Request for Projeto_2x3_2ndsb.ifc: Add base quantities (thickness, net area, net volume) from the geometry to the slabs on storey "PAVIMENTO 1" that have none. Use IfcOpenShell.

First a look at what the model holds.

```python
import ifcopenshell
import ifcopenshell.util.element
import ifcopenshell.util.unit

model = ifcopenshell.open("Projeto_2x3_2ndsb.ifc")
print(model.schema)
for unit_type in ("LENGTHUNIT", "AREAUNIT", "VOLUMEUNIT"):
    print(unit_type, ifcopenshell.util.unit.calculate_unit_scale(model, unit_type))
storey = next(s for s in model.by_type("IfcBuildingStorey") if s.Name == "PAVIMENTO 1")
slabs = [e for e in ifcopenshell.util.element.get_decomposition(storey) if e.is_a("IfcSlab")]
for e in sorted(slabs, key=lambda e: e.id()):
    print(e.id(), e.is_a(), e.Name, list(ifcopenshell.util.element.get_psets(e, qtos_only=True)), sep=" | ")
```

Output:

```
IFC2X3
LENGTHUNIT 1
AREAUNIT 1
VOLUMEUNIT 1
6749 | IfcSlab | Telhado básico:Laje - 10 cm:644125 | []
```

```python
import ifcopenshell
import ifcopenshell.api.pset
import ifcopenshell.geom
import ifcopenshell.util.element
import ifcopenshell.util.shape
import ifcopenshell.util.unit

model = ifcopenshell.open("Projeto_2x3_2ndsb.ifc")
unit_scale = ifcopenshell.util.unit.calculate_unit_scale(model)
area_scale = ifcopenshell.util.unit.calculate_unit_scale(model, "AREAUNIT")
volume_scale = ifcopenshell.util.unit.calculate_unit_scale(model, "VOLUMEUNIT")
settings = ifcopenshell.geom.settings()

storey = next(s for s in model.by_type("IfcBuildingStorey") if s.Name == "PAVIMENTO 1")
slabs = [e for e in ifcopenshell.util.element.get_decomposition(storey) if e.is_a("IfcSlab")]

for e in sorted(slabs, key=lambda e: e.id()):
    if ifcopenshell.util.element.get_psets(e, qtos_only=True, should_inherit=False):
        continue
    # Geometry comes back in metres, in the element's own axes.
    shape = ifcopenshell.geom.create_shape(settings, e)
    values = {
        "Width": ifcopenshell.util.shape.get_z(shape.geometry) / unit_scale,
        "NetArea": ifcopenshell.util.shape.get_footprint_area(shape.geometry) / area_scale,
        "NetVolume": ifcopenshell.util.shape.get_volume(shape.geometry) / volume_scale,
    }
    qto = ifcopenshell.api.pset.add_qto(model, product=e, name="BaseQuantities")
    ifcopenshell.api.pset.edit_qto(model, qto=qto, properties=values)
    print(e.id(), {k: round(v, 3) for k, v in values.items()})

model.write("Projeto_2x3_2ndsb-out.ifc")
```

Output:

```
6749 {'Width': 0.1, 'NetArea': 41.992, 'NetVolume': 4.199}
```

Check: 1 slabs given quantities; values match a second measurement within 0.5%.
